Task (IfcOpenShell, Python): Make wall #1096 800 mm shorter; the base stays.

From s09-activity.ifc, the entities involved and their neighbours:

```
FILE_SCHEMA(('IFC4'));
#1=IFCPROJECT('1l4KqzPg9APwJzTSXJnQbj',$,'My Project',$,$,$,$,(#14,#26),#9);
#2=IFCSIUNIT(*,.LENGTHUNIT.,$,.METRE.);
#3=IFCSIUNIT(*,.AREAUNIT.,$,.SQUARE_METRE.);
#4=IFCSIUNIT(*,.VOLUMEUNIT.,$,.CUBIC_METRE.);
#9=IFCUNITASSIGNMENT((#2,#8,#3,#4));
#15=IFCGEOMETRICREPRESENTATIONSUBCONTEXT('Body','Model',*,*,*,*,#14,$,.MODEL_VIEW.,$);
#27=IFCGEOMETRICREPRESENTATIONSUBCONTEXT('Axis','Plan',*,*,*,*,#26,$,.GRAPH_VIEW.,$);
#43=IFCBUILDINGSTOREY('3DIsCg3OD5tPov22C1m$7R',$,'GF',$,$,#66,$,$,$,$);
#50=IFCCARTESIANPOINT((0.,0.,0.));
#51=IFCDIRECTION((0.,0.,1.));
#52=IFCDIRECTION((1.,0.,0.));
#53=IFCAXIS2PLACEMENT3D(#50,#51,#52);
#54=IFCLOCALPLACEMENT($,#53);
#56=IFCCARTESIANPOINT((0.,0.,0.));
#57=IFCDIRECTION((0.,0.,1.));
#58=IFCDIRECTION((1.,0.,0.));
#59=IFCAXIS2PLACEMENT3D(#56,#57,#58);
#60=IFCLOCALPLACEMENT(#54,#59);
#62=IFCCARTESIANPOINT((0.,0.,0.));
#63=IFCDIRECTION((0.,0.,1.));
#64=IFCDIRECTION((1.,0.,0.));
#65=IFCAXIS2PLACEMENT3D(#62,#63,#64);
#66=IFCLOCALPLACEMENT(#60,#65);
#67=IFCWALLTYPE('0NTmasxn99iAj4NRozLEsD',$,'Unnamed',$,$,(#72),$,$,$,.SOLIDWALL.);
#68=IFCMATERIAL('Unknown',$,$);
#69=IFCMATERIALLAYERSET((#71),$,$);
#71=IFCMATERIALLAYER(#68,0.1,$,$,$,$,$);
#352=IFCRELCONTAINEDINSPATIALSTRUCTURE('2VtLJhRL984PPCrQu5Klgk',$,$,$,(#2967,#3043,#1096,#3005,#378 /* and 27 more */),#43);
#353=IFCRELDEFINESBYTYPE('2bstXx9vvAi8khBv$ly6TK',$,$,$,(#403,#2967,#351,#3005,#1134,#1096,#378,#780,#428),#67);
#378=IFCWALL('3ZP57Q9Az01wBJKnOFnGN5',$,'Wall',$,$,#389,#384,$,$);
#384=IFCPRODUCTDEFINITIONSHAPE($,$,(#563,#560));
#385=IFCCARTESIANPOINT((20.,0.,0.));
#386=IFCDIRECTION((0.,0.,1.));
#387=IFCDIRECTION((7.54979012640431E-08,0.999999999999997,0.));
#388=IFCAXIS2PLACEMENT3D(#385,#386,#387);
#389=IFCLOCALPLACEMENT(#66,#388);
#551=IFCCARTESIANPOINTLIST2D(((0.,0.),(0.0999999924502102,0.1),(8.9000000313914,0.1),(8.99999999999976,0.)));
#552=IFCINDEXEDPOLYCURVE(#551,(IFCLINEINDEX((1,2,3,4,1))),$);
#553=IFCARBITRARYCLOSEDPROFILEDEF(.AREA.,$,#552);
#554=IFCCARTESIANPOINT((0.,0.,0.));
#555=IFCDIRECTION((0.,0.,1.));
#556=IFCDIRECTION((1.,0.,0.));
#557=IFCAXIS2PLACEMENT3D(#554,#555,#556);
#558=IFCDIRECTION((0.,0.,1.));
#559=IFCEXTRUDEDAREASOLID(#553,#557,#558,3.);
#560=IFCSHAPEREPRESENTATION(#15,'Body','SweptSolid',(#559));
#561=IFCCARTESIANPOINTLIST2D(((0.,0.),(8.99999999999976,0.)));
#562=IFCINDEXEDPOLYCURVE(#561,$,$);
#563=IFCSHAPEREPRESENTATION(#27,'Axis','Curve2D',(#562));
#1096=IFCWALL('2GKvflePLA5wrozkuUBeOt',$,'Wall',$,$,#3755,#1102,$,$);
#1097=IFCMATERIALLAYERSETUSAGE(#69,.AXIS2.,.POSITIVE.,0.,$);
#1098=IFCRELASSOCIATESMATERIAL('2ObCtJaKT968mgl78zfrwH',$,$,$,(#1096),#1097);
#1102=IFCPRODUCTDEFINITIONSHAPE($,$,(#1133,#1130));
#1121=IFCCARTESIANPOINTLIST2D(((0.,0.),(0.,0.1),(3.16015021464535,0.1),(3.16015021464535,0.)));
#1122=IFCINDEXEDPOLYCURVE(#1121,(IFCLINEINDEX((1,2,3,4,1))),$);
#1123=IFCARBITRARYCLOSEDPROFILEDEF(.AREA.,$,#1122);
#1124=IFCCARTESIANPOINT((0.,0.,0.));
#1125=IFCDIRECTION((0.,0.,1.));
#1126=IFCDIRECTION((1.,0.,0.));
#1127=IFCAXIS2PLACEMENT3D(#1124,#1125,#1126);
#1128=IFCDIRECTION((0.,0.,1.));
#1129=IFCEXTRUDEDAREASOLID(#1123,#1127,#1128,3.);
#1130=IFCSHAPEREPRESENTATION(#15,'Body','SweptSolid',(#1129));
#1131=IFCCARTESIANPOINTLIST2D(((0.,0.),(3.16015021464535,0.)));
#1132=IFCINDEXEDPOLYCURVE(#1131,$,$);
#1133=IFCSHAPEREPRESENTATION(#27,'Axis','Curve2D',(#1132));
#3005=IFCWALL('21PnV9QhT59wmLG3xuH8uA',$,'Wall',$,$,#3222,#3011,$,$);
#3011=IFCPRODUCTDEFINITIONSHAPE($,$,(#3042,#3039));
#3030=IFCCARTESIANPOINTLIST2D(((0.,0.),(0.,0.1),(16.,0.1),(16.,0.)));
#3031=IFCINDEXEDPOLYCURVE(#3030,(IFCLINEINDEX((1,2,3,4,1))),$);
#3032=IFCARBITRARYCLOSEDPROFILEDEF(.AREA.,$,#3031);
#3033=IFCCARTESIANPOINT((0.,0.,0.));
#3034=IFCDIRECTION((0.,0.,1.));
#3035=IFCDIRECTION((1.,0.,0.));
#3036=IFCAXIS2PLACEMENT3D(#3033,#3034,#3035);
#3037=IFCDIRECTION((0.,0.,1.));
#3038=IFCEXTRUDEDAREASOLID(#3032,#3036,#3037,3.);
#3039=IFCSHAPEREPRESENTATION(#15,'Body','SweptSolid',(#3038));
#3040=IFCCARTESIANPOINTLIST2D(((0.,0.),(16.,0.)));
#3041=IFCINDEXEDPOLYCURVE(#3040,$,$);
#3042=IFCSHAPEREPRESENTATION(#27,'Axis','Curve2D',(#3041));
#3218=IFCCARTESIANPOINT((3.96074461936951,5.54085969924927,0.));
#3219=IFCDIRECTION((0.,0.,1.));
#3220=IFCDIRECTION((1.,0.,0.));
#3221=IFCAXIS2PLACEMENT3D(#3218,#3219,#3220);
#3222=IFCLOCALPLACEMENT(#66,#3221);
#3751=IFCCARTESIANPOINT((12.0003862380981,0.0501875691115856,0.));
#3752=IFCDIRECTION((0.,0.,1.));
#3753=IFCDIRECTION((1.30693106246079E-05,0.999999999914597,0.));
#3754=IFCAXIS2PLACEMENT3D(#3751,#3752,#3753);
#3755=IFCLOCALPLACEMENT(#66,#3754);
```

```python
import ifcopenshell
import ifcopenshell.geom
import ifcopenshell.util.representation
import ifcopenshell.util.shape
import ifcopenshell.util.unit

model = ifcopenshell.open("s09-activity.ifc")
unit_scale = ifcopenshell.util.unit.calculate_unit_scale(model)
settings = ifcopenshell.geom.settings()


def volume(element):
    """Net volume in cubic metres, openings subtracted."""
    shape = ifcopenshell.geom.create_shape(settings, element)
    return ifcopenshell.util.shape.get_volume(shape.geometry)


wall = model.by_guid("2GKvflePLA5wrozkuUBeOt")
before = volume(wall)

body = ifcopenshell.util.representation.get_representation(wall, "Model", "Body")
solid = body.Items[0]
old_height = solid.Depth
solid.Depth -= 0.8 / unit_scale
after = volume(wall)

print(f"height {old_height:g} -> {solid.Depth:g}, volume {before:.3f} -> {after:.3f} m3")

model.write("s09-activity_edited.ifc")
```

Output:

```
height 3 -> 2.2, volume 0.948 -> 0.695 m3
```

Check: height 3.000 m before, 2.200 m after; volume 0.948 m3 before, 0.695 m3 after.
